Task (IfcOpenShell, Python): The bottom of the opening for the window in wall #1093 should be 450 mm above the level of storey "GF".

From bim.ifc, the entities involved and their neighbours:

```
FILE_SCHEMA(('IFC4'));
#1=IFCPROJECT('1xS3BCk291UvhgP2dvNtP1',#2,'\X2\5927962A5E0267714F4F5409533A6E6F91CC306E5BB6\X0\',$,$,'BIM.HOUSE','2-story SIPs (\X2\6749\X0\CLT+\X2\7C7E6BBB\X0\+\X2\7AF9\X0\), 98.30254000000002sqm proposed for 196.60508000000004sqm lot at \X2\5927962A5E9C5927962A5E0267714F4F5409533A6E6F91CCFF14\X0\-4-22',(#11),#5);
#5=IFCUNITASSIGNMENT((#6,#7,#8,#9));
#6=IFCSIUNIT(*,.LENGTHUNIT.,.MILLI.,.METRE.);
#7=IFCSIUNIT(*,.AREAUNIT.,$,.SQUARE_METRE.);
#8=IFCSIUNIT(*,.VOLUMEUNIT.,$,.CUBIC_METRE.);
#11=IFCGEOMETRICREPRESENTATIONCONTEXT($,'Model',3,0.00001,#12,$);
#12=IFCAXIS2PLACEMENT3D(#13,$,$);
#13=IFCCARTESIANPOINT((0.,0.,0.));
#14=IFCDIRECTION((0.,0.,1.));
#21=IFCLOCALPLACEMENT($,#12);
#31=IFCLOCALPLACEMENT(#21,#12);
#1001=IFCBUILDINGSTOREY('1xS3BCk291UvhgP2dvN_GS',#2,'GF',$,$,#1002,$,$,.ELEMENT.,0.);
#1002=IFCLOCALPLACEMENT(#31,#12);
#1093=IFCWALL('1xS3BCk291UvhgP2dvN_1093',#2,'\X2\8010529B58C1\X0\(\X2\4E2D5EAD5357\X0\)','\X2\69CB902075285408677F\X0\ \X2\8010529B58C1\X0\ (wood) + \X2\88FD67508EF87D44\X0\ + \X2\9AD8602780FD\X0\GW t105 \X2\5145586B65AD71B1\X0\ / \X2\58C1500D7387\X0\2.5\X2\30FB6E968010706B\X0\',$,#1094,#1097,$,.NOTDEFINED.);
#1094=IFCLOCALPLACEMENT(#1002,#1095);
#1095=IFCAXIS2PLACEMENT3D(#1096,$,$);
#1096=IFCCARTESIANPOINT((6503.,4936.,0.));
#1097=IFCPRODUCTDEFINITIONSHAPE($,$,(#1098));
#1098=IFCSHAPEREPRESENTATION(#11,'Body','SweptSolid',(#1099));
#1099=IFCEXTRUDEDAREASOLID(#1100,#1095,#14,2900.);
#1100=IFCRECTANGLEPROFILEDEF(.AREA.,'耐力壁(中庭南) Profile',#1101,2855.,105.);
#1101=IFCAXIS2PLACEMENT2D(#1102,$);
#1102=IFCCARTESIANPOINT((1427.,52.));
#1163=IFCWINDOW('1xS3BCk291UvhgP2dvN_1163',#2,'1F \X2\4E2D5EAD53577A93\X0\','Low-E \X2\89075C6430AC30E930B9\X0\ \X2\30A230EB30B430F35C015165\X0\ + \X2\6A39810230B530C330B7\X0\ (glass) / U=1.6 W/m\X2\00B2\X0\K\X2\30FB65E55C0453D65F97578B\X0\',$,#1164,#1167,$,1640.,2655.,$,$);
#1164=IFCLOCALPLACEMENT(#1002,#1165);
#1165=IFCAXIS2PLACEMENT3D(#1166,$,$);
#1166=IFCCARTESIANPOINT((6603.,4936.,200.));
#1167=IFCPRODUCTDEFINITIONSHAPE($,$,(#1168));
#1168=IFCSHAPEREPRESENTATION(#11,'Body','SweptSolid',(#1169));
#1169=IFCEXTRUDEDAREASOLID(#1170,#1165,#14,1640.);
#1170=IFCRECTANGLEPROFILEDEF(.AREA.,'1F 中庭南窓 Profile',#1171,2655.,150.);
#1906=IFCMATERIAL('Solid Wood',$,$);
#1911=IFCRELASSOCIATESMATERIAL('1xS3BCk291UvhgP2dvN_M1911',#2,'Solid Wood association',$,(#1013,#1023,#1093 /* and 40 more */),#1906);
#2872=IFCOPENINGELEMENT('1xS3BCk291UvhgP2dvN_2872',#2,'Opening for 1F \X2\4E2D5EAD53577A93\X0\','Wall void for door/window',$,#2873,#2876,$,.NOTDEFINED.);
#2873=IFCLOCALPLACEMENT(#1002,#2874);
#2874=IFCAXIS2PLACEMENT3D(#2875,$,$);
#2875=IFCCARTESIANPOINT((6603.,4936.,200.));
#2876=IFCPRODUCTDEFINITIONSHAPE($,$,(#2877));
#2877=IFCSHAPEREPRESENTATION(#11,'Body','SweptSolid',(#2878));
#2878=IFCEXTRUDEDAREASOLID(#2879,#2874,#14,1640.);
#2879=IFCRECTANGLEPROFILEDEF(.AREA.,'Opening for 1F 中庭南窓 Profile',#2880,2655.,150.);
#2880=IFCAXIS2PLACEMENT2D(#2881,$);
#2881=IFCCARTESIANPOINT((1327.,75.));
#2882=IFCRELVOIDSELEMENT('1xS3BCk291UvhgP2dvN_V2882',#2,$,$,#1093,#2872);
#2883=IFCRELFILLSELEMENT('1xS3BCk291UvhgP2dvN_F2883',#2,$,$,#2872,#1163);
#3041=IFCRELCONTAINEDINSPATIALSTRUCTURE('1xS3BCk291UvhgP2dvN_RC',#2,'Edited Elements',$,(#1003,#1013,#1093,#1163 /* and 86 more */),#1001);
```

```python
import numpy as np
import ifcopenshell
import ifcopenshell.api.geometry
import ifcopenshell.geom
import ifcopenshell.util.element
import ifcopenshell.util.placement
import ifcopenshell.util.shape
import ifcopenshell.util.unit

model = ifcopenshell.open("bim.ifc")
unit_scale = ifcopenshell.util.unit.calculate_unit_scale(model)

window = model.by_guid("1xS3BCk291UvhgP2dvN_1163")
opening = window.FillsVoids[0].RelatingOpeningElement
storey = ifcopenshell.util.element.get_container(window, ifc_class="IfcBuildingStorey")
level = ifcopenshell.util.placement.get_local_placement(storey.ObjectPlacement)[2, 3]

# The opening's origin need not be at the sill, so measure its lowest point.
shape = ifcopenshell.geom.create_shape(ifcopenshell.geom.settings(), opening)
bottom = ifcopenshell.util.shape.get_shape_bottom_elevation(shape, shape.geometry) / unit_scale
dz = level + 0.45 / unit_scale - bottom

shift = np.array([0.0, 0.0, dz])
# The window is not placed relative to its opening, so move both.
for product in (opening, window):
    matrix = ifcopenshell.util.placement.get_local_placement(product.ObjectPlacement)
    matrix[:3, 3] += shift
    ifcopenshell.api.geometry.edit_object_placement(model, product=product, matrix=matrix, is_si=False)

print(f"moved by {dz * unit_scale:+.3f} m")

model.write("bim_updated.ifc")
```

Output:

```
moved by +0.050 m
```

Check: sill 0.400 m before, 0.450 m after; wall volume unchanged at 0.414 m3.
